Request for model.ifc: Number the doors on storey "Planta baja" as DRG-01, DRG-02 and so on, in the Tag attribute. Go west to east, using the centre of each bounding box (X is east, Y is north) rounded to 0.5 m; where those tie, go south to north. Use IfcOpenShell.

First a look at what the model holds.

```python
import ifcopenshell
import ifcopenshell.util.element
import ifcopenshell.util.placement

model = ifcopenshell.open("model.ifc")
print(model.schema)
storey = next(s for s in model.by_type("IfcBuildingStorey") if s.Name == "Planta baja")
doors = [e for e in ifcopenshell.util.element.get_decomposition(storey) if e.is_a("IfcDoor")]
for e in sorted(doors, key=lambda e: e.id()):
    origin = ifcopenshell.util.placement.get_local_placement(e.ObjectPlacement)[:3, 3]
    print(e.id(), e.Tag, e.Name, origin.round(2) + 0.0, sep=" | ")
```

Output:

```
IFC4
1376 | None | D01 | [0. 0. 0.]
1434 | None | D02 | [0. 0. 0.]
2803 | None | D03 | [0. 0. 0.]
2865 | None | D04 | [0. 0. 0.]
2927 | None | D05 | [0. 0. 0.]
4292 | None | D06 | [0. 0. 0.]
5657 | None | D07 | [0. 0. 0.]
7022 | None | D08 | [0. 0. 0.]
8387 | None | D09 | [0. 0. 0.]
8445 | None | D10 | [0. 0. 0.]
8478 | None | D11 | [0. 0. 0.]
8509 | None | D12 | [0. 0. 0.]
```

```python
import ifcopenshell
import ifcopenshell.geom
import ifcopenshell.util.element
import ifcopenshell.util.shape

model = ifcopenshell.open("model.ifc")
settings = ifcopenshell.geom.settings()
settings.set("use-world-coords", True)


def centre(element):
    shape = ifcopenshell.geom.create_shape(settings, element)
    return ifcopenshell.util.shape.get_bbox_centroid(shape.geometry)


storey = next(s for s in model.by_type("IfcBuildingStorey") if s.Name == "Planta baja")
doors = [e for e in ifcopenshell.util.element.get_decomposition(storey) if e.is_a("IfcDoor")]

# Insertion points can sit at a corner or the storey origin, so sort by the geometry (in metres).
centres = {e: centre(e) for e in doors}
doors.sort(key=lambda e: (round(centres[e][0] / 0.5), centres[e][1]))

for i, e in enumerate(doors, start=1):
    number = f"DRG-{i:02d}"
    e.Tag = number
    print(e.id(), number)

model.write("model_rev.ifc")
```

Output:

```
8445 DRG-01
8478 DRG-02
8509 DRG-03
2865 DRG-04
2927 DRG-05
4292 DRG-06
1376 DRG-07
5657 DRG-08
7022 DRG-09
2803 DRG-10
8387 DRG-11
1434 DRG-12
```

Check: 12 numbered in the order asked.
